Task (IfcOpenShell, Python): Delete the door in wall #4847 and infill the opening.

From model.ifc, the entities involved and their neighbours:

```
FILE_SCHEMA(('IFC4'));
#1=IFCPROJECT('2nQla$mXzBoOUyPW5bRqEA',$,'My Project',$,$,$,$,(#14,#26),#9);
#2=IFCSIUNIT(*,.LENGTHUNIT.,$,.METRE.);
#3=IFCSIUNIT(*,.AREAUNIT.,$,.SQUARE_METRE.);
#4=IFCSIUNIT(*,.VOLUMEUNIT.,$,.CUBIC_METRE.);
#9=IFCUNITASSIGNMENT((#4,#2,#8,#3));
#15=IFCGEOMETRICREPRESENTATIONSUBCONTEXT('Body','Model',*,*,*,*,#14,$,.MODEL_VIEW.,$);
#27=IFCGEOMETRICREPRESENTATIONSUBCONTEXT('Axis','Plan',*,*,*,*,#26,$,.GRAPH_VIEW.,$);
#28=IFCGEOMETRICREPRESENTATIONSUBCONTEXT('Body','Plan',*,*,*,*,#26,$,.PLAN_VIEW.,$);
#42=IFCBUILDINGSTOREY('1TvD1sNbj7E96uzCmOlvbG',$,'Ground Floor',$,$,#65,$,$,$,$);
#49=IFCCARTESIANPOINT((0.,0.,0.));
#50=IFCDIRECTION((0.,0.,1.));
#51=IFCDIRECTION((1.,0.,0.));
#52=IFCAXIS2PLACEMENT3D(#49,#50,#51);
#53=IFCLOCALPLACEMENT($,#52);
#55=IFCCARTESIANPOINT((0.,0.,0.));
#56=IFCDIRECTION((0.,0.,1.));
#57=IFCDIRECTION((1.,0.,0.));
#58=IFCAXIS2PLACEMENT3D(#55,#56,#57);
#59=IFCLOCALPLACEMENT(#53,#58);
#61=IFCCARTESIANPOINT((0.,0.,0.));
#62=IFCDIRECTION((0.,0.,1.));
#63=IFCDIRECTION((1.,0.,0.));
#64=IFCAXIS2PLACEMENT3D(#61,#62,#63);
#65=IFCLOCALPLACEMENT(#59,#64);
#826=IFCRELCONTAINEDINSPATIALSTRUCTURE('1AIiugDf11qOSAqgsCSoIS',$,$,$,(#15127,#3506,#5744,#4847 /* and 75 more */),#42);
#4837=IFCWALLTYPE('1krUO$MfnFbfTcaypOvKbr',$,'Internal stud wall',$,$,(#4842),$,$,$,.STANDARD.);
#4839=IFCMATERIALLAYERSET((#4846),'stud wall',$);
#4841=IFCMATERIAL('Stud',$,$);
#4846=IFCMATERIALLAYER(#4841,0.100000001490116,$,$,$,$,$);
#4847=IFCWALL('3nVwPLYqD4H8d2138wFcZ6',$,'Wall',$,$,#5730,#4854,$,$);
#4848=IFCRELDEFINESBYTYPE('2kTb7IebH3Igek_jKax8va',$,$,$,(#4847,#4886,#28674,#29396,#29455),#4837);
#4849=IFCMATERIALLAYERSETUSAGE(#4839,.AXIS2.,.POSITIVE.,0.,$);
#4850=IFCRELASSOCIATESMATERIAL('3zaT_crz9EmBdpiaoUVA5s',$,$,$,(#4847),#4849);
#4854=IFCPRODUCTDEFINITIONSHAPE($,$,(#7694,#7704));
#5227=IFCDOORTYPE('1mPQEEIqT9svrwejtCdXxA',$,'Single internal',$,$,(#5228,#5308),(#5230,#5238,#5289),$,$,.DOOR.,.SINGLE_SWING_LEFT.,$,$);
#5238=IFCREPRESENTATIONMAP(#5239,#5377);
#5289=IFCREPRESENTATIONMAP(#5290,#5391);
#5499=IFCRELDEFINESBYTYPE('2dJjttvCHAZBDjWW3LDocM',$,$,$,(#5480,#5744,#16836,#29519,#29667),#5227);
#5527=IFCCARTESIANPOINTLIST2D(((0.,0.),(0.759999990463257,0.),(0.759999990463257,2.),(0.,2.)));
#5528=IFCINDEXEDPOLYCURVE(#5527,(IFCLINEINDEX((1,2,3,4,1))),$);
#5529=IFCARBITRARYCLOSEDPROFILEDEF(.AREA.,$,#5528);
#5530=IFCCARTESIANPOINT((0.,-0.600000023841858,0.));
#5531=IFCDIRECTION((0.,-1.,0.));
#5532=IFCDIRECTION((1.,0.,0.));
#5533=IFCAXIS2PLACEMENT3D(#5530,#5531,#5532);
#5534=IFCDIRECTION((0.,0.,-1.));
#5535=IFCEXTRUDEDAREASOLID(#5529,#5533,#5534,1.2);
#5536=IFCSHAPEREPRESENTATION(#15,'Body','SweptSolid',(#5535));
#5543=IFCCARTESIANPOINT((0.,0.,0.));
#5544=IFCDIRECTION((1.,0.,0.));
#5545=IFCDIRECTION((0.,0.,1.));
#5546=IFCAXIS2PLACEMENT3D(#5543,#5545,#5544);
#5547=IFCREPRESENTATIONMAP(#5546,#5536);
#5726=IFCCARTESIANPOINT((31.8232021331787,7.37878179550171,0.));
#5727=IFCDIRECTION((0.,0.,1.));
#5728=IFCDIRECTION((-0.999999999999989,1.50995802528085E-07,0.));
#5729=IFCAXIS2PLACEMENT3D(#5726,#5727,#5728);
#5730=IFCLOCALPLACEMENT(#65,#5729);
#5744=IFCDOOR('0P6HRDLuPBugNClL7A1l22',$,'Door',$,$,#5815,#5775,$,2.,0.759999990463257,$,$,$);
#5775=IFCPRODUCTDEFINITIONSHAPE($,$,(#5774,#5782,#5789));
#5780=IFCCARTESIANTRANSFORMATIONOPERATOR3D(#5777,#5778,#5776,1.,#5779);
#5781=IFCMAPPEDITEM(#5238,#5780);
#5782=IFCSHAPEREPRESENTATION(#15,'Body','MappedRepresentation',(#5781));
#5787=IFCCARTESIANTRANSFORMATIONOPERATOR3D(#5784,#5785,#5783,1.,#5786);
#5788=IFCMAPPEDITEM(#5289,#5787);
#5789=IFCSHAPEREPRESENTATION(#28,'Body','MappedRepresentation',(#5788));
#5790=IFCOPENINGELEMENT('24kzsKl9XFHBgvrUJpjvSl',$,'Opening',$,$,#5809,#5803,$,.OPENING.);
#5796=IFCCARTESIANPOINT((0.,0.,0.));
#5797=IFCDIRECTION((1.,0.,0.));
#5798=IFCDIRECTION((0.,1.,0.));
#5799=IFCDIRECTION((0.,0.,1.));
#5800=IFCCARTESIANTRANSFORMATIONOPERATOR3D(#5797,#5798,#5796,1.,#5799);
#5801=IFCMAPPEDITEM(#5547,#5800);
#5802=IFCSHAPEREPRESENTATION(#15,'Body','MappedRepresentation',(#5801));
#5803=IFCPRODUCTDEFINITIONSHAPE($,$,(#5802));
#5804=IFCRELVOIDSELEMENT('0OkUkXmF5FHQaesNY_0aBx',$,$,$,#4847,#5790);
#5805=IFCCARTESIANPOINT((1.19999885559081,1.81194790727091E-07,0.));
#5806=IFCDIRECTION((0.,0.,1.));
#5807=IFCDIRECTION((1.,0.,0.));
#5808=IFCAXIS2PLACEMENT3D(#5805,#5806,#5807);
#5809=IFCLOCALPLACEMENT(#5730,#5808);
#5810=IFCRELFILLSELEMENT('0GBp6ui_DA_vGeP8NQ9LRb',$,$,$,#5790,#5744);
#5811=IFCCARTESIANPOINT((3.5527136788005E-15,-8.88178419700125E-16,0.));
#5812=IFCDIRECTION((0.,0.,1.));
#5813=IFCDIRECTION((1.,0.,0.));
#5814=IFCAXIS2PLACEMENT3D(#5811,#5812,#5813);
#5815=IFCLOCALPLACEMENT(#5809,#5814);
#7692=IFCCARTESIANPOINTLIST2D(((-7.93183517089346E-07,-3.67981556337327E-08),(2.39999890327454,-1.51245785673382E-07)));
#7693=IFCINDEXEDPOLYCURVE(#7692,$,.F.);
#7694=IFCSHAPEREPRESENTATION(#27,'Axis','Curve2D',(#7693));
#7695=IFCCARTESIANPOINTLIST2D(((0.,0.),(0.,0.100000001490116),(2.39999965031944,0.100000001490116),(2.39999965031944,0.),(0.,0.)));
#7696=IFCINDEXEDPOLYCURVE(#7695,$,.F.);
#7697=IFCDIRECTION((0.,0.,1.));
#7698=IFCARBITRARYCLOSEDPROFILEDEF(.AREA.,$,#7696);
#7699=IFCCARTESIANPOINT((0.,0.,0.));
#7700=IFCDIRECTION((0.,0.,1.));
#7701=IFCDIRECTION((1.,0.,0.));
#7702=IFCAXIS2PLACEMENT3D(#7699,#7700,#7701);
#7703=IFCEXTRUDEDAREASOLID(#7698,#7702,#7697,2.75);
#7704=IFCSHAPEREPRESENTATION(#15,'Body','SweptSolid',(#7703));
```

```python
import ifcopenshell
import ifcopenshell.api.feature
import ifcopenshell.api.root
import ifcopenshell.geom
import ifcopenshell.util.shape

model = ifcopenshell.open("model.ifc")
settings = ifcopenshell.geom.settings()


def volume(element):
    """Net volume in cubic metres, openings subtracted."""
    shape = ifcopenshell.geom.create_shape(settings, element)
    return ifcopenshell.util.shape.get_volume(shape.geometry)


door = model.by_guid("0P6HRDLuPBugNClL7A1l22")
opening = door.FillsVoids[0].RelatingOpeningElement
wall = opening.VoidsElements[0].RelatingBuildingElement
before = volume(wall)

ifcopenshell.api.root.remove_product(model, product=door)
ifcopenshell.api.feature.remove_feature(model, feature=opening)

after = volume(wall)

print(f"wall volume {before:.3f} -> {after:.3f} m3")

model.write("model_edited.ifc")
```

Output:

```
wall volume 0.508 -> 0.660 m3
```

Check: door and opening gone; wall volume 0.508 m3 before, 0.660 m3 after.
